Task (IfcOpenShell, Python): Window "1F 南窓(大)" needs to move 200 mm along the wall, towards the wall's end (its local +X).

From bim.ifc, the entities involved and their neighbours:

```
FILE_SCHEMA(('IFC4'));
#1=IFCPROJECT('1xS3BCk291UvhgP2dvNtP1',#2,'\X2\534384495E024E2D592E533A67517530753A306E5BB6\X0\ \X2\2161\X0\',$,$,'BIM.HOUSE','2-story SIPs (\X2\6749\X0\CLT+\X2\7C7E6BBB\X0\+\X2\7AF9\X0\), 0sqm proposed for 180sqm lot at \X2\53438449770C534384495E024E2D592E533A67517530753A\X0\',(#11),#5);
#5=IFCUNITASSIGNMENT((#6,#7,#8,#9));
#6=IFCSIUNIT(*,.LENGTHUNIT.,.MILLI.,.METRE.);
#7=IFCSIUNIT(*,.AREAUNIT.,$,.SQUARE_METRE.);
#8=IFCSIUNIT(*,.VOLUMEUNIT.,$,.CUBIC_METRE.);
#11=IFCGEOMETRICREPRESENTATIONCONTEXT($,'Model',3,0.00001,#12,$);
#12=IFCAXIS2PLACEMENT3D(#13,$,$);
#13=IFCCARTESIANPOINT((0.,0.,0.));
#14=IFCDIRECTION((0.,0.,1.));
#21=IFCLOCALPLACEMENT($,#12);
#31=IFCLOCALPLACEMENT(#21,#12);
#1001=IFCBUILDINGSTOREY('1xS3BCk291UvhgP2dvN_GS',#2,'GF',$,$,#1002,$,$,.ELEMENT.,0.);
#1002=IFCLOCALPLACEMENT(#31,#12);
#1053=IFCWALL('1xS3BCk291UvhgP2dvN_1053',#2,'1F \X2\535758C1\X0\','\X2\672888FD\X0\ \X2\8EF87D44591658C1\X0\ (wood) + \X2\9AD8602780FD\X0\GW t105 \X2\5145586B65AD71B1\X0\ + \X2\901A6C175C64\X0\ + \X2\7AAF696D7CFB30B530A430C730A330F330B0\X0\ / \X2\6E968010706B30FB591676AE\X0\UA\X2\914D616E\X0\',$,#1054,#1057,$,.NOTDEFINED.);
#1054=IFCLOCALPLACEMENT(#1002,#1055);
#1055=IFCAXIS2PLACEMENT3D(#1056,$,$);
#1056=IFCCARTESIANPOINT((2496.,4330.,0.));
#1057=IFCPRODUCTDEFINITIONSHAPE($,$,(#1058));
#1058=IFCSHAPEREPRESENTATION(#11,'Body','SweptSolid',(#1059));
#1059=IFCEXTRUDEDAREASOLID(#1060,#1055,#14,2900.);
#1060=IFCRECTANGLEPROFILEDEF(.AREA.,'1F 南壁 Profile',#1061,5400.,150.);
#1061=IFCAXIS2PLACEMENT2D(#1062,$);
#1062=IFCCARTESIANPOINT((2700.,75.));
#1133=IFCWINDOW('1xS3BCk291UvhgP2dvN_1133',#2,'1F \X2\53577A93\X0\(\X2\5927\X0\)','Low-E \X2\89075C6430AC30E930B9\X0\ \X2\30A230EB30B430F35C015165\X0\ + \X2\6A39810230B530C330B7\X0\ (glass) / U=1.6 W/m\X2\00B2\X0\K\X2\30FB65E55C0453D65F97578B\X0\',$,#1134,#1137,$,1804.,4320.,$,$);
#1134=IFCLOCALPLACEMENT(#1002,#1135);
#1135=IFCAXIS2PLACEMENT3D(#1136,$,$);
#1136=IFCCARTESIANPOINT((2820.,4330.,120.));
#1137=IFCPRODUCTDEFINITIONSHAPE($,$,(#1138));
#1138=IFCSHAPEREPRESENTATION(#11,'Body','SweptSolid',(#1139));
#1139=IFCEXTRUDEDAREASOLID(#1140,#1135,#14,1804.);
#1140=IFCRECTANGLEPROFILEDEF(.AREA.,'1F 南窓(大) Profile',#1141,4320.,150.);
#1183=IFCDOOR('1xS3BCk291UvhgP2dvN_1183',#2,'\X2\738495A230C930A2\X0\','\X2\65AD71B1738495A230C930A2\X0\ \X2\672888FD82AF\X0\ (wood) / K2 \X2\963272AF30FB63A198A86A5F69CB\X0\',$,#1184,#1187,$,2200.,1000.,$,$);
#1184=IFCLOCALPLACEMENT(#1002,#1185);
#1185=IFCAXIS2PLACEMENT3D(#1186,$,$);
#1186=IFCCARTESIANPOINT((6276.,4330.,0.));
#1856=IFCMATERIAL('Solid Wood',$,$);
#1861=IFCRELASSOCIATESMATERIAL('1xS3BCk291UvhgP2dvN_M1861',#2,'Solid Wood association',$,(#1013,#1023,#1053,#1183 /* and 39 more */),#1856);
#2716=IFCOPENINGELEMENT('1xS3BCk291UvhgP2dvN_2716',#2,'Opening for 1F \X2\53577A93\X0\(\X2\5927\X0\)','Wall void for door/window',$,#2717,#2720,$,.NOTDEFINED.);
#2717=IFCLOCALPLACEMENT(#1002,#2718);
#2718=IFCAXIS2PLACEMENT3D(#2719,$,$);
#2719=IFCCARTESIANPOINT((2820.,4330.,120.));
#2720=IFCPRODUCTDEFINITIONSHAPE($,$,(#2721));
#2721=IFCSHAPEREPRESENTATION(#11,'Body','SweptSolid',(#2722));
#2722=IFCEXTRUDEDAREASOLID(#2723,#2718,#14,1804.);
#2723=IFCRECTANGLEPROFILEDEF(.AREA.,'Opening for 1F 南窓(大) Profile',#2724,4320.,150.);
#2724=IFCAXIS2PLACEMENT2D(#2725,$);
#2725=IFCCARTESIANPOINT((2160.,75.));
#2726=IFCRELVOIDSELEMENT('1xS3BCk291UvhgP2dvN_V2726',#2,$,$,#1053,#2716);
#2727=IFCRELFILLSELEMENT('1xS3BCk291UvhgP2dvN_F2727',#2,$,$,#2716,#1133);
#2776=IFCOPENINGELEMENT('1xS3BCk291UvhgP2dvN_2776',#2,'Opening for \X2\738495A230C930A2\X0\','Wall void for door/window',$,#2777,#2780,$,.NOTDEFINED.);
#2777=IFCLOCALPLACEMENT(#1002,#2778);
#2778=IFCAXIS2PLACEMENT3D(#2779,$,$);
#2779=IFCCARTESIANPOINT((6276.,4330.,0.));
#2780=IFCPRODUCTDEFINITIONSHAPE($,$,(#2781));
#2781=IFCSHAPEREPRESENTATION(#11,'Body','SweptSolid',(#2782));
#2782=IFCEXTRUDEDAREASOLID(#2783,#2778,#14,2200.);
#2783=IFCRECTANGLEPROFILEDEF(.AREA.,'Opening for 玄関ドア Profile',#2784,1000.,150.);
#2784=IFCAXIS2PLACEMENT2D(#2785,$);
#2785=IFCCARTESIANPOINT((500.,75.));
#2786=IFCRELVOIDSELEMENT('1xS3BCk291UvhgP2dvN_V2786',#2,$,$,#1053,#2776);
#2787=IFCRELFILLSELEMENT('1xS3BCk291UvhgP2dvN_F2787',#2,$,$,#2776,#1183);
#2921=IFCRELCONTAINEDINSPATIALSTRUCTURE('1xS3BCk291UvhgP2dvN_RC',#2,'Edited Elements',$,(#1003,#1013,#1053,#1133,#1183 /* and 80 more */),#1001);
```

```python
import ifcopenshell
import ifcopenshell.api.geometry
import ifcopenshell.util.placement

model = ifcopenshell.open("bim.ifc")

window = model.by_guid("1xS3BCk291UvhgP2dvN_1133")
opening = window.FillsVoids[0].RelatingOpeningElement
wall = opening.VoidsElements[0].RelatingBuildingElement

wall_matrix = ifcopenshell.util.placement.get_local_placement(wall.ObjectPlacement)
shift = wall_matrix[:3, 0] * 200.0
before = ifcopenshell.util.placement.get_local_placement(window.ObjectPlacement)[:3, 3].copy()

# The window is not placed relative to its opening, so move both.
for product in (opening, window):
    matrix = ifcopenshell.util.placement.get_local_placement(product.ObjectPlacement)
    matrix[:3, 3] += shift
    ifcopenshell.api.geometry.edit_object_placement(model, product=product, matrix=matrix, is_si=False)

after = ifcopenshell.util.placement.get_local_placement(window.ObjectPlacement)[:3, 3]
print("window moved by", (after - before).round(3) + 0.0)

model.write("bim_updated.ifc")
```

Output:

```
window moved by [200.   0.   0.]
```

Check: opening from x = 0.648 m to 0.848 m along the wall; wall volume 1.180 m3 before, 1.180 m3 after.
